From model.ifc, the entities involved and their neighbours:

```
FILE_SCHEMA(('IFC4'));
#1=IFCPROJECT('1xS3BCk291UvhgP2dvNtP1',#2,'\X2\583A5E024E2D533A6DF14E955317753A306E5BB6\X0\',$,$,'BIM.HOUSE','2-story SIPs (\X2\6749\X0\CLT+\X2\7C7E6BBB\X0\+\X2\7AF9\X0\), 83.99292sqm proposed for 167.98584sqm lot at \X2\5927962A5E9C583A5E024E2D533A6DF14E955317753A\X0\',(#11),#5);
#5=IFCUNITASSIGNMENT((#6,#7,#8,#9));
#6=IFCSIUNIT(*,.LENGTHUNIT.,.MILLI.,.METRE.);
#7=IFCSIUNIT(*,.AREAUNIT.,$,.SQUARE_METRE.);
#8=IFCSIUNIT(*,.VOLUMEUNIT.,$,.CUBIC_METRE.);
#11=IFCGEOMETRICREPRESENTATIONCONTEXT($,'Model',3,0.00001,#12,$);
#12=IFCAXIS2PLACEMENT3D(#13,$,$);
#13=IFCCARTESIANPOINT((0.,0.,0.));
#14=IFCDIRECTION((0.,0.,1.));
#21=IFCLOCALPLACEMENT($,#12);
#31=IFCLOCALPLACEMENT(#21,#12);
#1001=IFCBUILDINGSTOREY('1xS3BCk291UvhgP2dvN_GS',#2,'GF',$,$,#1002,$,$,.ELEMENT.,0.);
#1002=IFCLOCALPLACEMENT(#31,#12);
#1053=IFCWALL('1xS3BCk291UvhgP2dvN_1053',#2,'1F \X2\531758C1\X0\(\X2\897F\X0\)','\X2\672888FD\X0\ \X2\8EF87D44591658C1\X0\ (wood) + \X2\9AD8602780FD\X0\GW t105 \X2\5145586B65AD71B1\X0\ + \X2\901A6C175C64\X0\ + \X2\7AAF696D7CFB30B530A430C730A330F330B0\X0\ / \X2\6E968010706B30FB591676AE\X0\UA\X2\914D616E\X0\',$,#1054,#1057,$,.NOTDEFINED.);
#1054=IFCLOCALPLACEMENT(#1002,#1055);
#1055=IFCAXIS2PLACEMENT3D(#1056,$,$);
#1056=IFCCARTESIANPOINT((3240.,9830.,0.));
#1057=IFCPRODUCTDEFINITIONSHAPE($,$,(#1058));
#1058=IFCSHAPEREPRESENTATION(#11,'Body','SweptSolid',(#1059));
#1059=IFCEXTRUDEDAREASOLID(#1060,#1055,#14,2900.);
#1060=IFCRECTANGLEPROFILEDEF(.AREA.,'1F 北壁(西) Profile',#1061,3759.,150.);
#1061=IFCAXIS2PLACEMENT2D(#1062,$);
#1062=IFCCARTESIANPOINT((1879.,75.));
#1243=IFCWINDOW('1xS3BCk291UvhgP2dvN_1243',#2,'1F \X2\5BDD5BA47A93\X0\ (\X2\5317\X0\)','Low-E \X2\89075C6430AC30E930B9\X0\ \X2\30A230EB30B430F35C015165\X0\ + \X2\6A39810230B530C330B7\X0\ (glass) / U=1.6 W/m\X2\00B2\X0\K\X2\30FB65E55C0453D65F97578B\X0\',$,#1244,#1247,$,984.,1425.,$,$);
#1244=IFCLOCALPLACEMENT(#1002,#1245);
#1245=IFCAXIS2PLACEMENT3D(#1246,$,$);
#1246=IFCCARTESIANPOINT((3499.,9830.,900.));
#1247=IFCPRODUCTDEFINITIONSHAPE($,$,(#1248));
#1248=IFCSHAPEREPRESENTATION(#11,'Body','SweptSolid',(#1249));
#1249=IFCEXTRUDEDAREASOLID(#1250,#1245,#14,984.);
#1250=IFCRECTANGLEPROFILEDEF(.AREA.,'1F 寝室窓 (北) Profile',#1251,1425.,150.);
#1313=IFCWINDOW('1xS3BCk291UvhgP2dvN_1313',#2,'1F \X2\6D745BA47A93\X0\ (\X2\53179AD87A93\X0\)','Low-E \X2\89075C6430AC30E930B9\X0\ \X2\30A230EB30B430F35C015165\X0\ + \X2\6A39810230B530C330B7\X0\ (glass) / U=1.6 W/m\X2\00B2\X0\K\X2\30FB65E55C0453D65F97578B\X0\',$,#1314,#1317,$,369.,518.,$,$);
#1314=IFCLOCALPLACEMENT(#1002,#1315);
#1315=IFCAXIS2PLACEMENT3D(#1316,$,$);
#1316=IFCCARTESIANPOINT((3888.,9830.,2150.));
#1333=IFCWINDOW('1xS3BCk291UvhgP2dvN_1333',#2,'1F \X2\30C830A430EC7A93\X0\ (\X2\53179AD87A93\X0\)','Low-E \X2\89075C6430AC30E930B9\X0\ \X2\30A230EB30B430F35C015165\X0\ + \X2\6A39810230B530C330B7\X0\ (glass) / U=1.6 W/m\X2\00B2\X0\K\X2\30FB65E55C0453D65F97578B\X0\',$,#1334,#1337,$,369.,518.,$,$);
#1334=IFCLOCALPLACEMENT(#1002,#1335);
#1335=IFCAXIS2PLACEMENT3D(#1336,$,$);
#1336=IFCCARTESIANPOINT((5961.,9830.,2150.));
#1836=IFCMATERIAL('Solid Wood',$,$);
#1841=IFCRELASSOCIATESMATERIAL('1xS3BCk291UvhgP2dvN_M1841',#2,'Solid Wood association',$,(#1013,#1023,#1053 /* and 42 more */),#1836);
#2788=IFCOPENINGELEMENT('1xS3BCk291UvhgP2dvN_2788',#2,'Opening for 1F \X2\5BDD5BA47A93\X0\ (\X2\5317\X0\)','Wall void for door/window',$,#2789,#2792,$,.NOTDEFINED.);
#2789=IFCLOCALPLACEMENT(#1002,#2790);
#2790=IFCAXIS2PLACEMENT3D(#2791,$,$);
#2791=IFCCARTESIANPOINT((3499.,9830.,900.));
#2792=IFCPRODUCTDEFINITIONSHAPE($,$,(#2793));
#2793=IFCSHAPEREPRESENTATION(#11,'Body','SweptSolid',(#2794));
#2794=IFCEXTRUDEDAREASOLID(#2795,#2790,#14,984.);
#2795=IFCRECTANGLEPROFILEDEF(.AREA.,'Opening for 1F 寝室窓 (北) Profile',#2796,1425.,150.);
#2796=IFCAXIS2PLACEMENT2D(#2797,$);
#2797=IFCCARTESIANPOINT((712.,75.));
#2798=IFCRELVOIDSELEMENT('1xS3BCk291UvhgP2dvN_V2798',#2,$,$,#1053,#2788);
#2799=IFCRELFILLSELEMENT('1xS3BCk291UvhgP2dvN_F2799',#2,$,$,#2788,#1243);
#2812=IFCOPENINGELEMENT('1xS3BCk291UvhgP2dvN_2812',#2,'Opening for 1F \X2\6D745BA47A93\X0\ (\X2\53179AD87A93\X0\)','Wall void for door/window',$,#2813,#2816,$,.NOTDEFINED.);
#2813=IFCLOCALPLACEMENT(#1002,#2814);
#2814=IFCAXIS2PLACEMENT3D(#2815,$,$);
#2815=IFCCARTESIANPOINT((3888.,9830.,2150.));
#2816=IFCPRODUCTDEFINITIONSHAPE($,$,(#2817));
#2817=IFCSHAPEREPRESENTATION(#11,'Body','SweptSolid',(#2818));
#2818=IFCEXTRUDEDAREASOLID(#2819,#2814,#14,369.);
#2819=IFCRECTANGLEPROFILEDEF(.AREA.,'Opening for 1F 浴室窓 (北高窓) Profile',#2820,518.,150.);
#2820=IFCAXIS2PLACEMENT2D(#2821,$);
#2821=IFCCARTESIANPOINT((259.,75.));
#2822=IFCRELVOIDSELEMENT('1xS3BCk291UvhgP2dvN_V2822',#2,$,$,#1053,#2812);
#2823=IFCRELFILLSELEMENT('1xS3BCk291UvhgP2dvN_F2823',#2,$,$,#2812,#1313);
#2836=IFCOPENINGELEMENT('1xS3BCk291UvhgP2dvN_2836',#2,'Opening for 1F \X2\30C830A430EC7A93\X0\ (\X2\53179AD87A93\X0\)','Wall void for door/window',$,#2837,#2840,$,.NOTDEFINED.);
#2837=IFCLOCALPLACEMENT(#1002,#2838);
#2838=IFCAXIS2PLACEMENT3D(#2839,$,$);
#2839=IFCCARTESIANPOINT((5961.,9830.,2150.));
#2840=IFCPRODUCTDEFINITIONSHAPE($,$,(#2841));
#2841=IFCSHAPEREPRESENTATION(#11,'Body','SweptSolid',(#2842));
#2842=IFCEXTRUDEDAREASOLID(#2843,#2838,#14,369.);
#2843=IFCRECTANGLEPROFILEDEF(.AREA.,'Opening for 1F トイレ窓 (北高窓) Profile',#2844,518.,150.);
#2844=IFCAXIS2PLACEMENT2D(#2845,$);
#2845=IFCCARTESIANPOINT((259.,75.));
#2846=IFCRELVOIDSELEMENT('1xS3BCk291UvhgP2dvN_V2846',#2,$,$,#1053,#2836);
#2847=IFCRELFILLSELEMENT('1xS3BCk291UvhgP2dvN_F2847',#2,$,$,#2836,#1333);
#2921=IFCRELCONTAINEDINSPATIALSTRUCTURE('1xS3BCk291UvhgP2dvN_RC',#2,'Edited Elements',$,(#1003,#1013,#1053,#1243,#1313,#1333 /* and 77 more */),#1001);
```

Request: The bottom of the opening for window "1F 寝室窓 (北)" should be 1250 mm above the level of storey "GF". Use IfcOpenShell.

```python
import numpy as np
import ifcopenshell
import ifcopenshell.api.geometry
import ifcopenshell.geom
import ifcopenshell.util.element
import ifcopenshell.util.placement
import ifcopenshell.util.shape
import ifcopenshell.util.unit

model = ifcopenshell.open("model.ifc")
unit_scale = ifcopenshell.util.unit.calculate_unit_scale(model)

window = model.by_guid("1xS3BCk291UvhgP2dvN_1243")
opening = window.FillsVoids[0].RelatingOpeningElement
storey = ifcopenshell.util.element.get_container(window, ifc_class="IfcBuildingStorey")
level = ifcopenshell.util.placement.get_local_placement(storey.ObjectPlacement)[2, 3]

# The opening's origin need not be at the sill, so measure its lowest point.
shape = ifcopenshell.geom.create_shape(ifcopenshell.geom.settings(), opening)
bottom = ifcopenshell.util.shape.get_shape_bottom_elevation(shape, shape.geometry) / unit_scale
dz = level + 1.25 / unit_scale - bottom

shift = np.array([0.0, 0.0, dz])
# The window is not placed relative to its opening, so move both.
for product in (opening, window):
    matrix = ifcopenshell.util.placement.get_local_placement(product.ObjectPlacement)
    matrix[:3, 3] += shift
    ifcopenshell.api.geometry.edit_object_placement(model, product=product, matrix=matrix, is_si=False)

print(f"moved by {dz * unit_scale:+.3f} m")

model.write("model_edited.ifc")
```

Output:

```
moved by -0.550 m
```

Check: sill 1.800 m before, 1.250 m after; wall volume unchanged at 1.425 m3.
